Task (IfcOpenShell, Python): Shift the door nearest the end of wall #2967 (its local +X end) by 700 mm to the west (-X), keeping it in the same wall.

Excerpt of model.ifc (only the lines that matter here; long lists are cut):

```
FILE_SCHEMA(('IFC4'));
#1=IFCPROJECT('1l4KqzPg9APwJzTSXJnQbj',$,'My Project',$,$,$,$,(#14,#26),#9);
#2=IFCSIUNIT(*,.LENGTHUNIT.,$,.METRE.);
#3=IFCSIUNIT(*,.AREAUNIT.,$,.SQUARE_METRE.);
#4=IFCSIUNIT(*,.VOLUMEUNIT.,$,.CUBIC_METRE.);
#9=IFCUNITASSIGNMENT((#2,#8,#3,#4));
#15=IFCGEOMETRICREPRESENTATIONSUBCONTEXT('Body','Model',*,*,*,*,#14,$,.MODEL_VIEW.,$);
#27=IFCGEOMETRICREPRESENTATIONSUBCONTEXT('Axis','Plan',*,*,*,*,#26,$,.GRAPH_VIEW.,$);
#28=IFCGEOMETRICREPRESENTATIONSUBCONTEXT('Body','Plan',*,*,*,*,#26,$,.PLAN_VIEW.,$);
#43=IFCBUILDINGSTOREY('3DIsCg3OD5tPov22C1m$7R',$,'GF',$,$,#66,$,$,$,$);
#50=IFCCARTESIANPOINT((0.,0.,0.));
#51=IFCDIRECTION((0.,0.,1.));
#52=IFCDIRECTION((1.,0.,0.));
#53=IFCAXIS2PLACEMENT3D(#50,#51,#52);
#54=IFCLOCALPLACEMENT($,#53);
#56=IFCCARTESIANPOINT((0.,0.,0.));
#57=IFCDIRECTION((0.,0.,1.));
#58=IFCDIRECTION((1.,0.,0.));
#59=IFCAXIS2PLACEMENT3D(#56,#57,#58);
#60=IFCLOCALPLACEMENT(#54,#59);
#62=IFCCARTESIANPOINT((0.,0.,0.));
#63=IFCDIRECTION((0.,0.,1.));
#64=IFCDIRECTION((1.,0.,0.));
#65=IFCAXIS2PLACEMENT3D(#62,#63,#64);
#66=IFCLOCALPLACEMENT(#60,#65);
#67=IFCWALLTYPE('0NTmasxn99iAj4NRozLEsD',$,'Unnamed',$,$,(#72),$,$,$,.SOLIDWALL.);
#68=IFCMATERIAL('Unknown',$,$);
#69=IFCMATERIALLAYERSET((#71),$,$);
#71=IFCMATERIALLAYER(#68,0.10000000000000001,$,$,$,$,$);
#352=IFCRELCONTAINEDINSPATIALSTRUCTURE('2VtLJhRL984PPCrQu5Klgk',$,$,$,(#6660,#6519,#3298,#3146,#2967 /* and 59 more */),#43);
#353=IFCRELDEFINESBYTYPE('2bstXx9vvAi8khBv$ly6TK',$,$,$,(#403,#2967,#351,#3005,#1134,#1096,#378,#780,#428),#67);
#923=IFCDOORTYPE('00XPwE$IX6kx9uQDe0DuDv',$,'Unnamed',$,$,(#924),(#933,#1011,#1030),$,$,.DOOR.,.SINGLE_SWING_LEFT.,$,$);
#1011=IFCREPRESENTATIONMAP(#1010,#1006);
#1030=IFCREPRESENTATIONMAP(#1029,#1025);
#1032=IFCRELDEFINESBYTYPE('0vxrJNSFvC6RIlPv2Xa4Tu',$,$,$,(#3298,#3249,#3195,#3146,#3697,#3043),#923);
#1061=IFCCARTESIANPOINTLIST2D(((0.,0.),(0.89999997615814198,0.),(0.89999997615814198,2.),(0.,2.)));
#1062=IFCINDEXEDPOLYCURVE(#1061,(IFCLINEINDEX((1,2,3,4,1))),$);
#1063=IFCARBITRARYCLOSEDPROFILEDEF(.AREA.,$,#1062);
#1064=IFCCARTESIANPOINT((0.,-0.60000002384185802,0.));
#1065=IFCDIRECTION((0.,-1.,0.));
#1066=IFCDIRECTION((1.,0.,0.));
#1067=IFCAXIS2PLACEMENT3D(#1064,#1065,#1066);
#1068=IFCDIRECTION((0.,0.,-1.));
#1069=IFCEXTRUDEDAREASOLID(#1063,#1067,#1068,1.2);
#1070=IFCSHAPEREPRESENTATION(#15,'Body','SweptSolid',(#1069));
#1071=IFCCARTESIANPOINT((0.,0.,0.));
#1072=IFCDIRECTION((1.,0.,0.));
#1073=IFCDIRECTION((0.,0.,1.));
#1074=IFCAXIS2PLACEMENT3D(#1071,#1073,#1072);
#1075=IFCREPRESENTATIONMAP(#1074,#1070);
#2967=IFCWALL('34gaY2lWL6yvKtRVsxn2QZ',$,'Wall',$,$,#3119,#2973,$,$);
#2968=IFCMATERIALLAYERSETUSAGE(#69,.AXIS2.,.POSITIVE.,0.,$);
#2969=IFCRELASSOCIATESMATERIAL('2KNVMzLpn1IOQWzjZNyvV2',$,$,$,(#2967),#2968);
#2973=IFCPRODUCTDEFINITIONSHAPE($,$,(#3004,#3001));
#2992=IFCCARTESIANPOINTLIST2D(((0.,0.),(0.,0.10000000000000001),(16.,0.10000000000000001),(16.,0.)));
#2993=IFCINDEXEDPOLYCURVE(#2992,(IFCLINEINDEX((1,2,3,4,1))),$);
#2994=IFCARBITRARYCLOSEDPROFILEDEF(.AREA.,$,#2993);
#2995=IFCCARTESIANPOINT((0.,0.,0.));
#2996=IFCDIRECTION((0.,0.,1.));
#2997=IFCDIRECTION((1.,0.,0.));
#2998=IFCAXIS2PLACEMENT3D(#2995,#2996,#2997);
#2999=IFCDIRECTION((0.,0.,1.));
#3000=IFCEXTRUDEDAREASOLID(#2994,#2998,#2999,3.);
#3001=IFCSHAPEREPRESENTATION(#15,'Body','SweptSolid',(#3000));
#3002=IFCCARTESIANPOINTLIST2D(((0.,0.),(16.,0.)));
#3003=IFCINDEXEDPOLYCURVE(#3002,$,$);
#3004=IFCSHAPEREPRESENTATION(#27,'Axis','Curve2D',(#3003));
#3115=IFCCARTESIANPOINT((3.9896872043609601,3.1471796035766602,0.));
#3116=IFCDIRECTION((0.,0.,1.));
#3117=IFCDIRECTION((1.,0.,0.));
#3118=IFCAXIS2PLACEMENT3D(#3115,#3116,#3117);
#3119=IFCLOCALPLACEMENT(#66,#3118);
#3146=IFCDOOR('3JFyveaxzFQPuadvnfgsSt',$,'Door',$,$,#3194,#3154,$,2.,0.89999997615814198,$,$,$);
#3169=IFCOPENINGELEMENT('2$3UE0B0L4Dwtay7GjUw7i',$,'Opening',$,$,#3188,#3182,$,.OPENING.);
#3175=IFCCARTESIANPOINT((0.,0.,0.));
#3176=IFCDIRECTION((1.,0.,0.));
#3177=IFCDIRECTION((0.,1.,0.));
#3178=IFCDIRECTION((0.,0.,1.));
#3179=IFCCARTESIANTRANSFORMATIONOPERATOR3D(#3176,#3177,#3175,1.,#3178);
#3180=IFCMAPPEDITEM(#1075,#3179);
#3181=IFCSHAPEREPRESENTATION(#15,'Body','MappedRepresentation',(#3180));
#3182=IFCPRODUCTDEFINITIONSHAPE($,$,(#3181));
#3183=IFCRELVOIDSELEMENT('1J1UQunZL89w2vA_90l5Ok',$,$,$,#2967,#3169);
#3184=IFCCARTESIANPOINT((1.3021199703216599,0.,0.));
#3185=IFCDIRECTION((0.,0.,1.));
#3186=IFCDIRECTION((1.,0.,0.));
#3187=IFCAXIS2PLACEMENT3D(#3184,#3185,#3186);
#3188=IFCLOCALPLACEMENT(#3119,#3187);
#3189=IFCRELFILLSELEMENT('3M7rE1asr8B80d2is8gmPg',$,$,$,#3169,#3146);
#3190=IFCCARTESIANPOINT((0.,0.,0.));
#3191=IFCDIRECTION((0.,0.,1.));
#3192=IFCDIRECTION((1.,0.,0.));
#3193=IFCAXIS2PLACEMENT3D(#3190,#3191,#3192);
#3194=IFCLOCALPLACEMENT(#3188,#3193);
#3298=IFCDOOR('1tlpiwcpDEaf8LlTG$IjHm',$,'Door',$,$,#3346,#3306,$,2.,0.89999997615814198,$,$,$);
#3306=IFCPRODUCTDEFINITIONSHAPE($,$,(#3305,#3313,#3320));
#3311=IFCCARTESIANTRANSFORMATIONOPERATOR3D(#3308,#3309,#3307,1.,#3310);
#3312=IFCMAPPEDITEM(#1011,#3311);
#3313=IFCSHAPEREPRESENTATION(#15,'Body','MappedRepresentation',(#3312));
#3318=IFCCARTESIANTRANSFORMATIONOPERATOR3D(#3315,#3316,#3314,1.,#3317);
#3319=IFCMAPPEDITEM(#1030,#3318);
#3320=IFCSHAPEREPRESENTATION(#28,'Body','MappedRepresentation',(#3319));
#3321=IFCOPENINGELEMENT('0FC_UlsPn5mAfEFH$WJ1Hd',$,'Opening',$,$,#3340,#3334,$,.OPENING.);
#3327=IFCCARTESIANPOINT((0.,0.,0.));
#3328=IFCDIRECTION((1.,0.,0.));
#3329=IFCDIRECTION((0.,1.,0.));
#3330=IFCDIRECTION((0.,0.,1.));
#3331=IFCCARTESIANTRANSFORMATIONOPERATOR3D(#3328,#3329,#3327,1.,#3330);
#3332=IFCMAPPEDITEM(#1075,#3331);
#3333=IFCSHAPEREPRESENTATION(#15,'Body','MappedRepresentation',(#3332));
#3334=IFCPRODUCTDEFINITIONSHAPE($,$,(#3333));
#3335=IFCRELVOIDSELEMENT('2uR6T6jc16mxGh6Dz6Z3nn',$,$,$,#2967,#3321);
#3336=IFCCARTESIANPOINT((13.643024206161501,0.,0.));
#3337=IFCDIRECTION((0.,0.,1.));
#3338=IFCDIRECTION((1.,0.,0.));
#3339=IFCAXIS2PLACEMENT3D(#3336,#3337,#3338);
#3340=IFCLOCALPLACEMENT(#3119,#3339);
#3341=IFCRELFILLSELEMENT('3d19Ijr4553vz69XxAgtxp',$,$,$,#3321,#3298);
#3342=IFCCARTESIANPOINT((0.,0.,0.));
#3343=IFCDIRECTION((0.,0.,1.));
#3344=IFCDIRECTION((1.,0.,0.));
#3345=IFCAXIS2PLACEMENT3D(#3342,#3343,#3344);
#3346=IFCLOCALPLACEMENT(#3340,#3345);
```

```python
import ifcopenshell
import ifcopenshell.api.geometry
import ifcopenshell.util.placement
import ifcopenshell.util.unit

model = ifcopenshell.open("model.ifc")
unit_scale = ifcopenshell.util.unit.calculate_unit_scale(model)

door = model.by_guid("1tlpiwcpDEaf8LlTG$IjHm")
opening = door.FillsVoids[0].RelatingOpeningElement
wall = opening.VoidsElements[0].RelatingBuildingElement

wall_matrix = ifcopenshell.util.placement.get_local_placement(wall.ObjectPlacement)
shift = wall_matrix[:3, 0] * -0.7 / unit_scale
before = ifcopenshell.util.placement.get_local_placement(door.ObjectPlacement)[:3, 3].copy()

# The door is placed relative to its opening, so it follows when the opening moves.
matrix = ifcopenshell.util.placement.get_local_placement(opening.ObjectPlacement)
matrix[:3, 3] += shift
ifcopenshell.api.geometry.edit_object_placement(
    model, product=opening, matrix=matrix, is_si=False, should_transform_children=True
)

after = ifcopenshell.util.placement.get_local_placement(door.ObjectPlacement)[:3, 3]
print("door moved by", (after - before).round(3) + 0.0)

model.write("model_v2.ifc")
```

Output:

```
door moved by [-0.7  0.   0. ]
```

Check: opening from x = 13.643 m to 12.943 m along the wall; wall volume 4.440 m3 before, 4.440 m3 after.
